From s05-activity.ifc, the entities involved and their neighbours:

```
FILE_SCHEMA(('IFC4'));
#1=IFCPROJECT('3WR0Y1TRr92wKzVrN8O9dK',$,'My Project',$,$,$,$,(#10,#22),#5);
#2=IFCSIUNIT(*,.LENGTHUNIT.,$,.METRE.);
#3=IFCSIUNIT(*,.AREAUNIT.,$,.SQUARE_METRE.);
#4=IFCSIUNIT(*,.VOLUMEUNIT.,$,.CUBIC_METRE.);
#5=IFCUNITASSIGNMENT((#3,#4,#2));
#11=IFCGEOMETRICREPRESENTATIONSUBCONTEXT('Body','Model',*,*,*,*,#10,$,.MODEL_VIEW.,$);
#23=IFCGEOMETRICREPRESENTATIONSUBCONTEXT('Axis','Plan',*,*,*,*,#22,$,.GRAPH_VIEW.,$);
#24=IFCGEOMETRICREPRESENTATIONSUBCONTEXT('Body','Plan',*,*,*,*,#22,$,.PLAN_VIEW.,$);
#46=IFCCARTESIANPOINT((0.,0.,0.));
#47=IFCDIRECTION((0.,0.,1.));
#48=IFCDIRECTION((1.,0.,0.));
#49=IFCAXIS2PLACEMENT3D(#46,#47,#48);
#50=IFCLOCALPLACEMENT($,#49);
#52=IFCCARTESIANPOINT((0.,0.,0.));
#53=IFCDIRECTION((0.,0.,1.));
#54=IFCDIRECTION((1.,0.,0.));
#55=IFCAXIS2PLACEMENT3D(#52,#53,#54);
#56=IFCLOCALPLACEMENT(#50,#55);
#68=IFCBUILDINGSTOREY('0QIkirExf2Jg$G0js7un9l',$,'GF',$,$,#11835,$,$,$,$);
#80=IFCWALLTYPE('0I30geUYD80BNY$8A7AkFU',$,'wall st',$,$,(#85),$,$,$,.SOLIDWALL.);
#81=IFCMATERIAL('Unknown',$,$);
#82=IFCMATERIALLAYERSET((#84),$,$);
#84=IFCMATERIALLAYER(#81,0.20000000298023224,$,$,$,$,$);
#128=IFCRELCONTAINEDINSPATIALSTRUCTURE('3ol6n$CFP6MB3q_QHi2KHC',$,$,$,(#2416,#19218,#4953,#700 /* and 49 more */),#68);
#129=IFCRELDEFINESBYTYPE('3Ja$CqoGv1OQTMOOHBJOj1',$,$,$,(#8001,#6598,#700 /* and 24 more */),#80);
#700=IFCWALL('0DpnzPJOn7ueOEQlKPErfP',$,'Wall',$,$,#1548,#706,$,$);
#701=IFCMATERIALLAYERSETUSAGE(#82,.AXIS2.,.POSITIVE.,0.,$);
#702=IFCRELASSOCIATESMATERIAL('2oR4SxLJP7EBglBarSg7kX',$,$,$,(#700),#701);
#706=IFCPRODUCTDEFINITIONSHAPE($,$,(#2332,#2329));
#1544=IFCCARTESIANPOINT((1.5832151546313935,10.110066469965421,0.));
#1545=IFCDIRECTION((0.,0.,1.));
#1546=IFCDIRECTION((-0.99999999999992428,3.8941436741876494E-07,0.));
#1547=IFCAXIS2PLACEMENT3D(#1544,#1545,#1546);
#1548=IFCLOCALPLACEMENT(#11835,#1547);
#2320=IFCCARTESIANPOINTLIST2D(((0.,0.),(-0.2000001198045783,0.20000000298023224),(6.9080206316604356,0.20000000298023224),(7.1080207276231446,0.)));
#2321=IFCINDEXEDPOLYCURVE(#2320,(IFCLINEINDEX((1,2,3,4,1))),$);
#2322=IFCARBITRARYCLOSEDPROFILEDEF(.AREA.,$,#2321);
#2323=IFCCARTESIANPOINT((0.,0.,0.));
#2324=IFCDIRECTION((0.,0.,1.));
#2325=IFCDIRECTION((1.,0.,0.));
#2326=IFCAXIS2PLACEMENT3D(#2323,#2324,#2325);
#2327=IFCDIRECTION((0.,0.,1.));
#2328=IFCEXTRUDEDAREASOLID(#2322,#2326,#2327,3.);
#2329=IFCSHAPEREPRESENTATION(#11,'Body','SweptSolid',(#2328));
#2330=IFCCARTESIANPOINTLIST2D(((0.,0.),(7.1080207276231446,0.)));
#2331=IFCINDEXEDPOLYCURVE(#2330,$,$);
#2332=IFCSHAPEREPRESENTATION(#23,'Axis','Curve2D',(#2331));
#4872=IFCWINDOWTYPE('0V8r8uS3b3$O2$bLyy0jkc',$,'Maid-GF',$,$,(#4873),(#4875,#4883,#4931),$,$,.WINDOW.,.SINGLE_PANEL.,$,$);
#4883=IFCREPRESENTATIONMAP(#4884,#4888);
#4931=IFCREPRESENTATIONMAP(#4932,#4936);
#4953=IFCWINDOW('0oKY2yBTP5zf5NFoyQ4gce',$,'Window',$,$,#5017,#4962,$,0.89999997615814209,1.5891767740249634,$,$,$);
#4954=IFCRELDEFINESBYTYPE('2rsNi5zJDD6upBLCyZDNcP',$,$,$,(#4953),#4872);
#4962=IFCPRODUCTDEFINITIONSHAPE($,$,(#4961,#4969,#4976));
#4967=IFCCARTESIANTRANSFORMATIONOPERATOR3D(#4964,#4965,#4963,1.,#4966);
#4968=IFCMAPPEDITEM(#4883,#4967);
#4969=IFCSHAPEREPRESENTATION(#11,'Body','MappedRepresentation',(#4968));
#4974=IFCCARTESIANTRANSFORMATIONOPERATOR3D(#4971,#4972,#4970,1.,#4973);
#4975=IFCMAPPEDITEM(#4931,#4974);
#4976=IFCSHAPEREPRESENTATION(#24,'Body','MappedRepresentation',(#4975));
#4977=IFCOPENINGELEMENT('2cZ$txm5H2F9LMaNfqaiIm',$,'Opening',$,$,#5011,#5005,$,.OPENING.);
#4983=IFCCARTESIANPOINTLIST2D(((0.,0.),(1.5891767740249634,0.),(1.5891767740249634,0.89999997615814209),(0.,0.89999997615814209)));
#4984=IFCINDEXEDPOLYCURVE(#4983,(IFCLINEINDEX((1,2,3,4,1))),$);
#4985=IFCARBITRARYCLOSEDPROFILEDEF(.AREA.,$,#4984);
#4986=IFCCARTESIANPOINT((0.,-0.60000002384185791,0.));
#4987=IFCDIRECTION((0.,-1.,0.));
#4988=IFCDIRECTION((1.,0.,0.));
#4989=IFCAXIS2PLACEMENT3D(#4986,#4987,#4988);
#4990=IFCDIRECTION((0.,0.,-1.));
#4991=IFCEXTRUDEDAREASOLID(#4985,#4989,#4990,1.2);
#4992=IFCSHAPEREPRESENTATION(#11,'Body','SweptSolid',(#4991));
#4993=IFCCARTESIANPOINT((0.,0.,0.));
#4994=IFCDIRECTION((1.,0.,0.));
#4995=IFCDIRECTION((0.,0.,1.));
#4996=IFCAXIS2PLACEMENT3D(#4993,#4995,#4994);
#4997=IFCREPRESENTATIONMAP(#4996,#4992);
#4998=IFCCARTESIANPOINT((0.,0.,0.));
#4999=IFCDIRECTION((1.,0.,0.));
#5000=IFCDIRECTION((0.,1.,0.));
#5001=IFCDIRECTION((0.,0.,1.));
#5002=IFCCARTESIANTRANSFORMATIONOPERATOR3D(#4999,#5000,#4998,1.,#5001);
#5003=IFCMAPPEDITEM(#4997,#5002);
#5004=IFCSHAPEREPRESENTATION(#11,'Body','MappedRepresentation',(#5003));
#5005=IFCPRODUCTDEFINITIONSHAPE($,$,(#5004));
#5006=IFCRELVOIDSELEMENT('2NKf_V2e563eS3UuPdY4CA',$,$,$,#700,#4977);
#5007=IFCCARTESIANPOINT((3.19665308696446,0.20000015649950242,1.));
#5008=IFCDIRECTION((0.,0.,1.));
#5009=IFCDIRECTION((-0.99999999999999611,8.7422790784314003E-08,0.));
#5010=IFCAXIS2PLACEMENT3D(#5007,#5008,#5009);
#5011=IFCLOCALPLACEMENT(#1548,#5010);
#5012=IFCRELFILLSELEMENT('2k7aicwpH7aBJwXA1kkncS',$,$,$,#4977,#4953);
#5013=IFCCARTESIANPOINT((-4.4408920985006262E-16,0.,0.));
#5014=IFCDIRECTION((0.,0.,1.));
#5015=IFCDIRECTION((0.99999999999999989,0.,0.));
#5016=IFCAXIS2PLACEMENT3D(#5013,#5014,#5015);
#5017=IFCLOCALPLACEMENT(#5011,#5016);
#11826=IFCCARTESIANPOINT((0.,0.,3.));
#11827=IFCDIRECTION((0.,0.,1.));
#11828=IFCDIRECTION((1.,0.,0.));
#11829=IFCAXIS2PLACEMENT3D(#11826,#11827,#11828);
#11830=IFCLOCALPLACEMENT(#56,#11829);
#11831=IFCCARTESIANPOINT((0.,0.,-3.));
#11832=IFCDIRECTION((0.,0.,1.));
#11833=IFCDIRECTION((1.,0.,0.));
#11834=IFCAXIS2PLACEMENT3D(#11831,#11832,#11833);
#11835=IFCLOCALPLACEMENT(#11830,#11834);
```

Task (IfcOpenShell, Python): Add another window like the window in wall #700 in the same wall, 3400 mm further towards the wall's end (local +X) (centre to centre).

```python
import ifcopenshell
import ifcopenshell.api.feature
import ifcopenshell.api.geometry
import ifcopenshell.api.root
import ifcopenshell.geom
import ifcopenshell.util.element
import ifcopenshell.util.placement
import ifcopenshell.util.shape

model = ifcopenshell.open("s05-activity.ifc")
settings = ifcopenshell.geom.settings()


def volume(element):
    """Net volume in cubic metres, openings subtracted."""
    shape = ifcopenshell.geom.create_shape(settings, element)
    return ifcopenshell.util.shape.get_volume(shape.geometry)


window = model.by_guid("0oKY2yBTP5zf5NFoyQ4gce")
opening = window.FillsVoids[0].RelatingOpeningElement
wall = opening.VoidsElements[0].RelatingBuildingElement
before = volume(wall)
shift = ifcopenshell.util.placement.get_local_placement(wall.ObjectPlacement)[:3, 0] * 3.4

# copy_class copies the void relationship, type, container and properties, but no geometry.
new_opening = ifcopenshell.api.root.copy_class(model, product=opening)
new_opening.Representation = ifcopenshell.util.element.copy_deep(
    model, opening.Representation, exclude=["IfcGeometricRepresentationContext", "IfcRepresentationMap"]
)
new_window = ifcopenshell.api.root.copy_class(model, product=window)
new_window.Representation = ifcopenshell.util.element.copy_deep(
    model, window.Representation, exclude=["IfcGeometricRepresentationContext", "IfcRepresentationMap"]
)
ifcopenshell.api.feature.add_filling(model, opening=new_opening, element=new_window)

for old, new in ((opening, new_opening), (window, new_window)):
    matrix = ifcopenshell.util.placement.get_local_placement(old.ObjectPlacement)
    matrix[:3, 3] += shift
    ifcopenshell.api.geometry.edit_object_placement(model, product=new, matrix=matrix, is_si=False)

after = volume(wall)

print(f"wall volume {before:.3f} -> {after:.3f} m3")

model.write("s05-activity_edited.ifc")
```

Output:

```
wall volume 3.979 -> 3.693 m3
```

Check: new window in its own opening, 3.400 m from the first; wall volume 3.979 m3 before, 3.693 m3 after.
